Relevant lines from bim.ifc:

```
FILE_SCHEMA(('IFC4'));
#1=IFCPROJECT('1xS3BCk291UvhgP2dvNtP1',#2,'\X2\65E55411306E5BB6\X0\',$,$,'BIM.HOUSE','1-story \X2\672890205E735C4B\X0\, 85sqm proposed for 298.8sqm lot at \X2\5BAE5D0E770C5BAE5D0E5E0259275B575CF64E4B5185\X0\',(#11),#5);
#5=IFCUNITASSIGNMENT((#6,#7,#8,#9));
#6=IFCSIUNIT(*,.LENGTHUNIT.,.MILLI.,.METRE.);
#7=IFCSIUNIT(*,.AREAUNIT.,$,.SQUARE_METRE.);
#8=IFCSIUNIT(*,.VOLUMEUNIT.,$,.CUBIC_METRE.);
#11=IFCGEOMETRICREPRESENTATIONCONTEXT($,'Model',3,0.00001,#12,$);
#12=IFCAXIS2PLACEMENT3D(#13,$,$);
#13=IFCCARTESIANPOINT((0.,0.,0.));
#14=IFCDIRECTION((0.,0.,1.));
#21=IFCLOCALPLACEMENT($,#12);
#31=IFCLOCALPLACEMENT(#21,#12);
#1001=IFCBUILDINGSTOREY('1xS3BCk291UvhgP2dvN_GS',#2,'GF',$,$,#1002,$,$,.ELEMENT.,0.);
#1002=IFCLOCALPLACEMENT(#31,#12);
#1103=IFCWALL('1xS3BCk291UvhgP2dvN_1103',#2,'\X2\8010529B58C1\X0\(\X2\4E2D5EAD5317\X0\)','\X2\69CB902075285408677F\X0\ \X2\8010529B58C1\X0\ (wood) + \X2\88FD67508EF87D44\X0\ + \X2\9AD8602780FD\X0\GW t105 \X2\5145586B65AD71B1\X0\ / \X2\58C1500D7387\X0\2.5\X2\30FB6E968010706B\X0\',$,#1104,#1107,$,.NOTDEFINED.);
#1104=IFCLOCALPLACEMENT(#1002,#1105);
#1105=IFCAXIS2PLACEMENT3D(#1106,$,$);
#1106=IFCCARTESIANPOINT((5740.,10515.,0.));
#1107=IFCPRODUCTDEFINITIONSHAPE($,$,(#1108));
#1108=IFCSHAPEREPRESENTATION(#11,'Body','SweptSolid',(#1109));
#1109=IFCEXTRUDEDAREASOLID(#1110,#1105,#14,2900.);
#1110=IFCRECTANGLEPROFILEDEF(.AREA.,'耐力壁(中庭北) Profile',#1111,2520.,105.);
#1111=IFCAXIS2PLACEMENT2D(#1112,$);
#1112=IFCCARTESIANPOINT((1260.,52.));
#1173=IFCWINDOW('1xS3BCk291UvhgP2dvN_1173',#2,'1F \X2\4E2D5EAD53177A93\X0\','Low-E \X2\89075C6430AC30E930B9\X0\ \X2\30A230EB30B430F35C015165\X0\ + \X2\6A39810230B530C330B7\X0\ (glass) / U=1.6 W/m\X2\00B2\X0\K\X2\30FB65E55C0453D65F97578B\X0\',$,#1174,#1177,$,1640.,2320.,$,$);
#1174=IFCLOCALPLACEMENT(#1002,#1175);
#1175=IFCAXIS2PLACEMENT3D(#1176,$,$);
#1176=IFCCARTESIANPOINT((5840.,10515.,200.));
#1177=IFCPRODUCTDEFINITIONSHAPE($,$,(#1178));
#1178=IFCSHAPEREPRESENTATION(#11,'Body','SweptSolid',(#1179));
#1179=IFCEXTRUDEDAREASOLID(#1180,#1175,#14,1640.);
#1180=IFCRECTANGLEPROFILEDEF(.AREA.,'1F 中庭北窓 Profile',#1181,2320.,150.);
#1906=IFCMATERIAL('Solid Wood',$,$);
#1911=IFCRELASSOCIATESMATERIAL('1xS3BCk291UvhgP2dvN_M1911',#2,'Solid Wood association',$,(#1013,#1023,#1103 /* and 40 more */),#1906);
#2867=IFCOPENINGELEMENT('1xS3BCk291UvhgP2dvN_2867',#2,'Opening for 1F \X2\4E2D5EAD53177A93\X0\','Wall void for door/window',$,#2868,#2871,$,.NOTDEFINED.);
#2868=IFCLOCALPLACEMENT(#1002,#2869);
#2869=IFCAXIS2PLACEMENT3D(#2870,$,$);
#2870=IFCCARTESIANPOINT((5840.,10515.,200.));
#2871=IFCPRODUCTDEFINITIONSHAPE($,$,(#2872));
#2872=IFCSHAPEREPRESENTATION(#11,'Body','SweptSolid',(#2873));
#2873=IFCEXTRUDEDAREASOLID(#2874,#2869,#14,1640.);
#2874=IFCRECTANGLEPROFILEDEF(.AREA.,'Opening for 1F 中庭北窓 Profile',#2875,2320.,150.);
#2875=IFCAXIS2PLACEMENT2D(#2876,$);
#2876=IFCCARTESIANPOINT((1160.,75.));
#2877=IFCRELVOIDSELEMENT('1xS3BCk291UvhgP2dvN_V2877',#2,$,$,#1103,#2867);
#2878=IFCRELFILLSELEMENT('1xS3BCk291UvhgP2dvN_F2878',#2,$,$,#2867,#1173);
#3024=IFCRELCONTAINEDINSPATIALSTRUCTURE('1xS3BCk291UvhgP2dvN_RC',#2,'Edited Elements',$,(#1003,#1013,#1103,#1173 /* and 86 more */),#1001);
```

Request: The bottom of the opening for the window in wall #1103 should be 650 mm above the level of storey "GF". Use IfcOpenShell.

```python
import numpy as np
import ifcopenshell
import ifcopenshell.api.geometry
import ifcopenshell.geom
import ifcopenshell.util.element
import ifcopenshell.util.placement
import ifcopenshell.util.shape
import ifcopenshell.util.unit

model = ifcopenshell.open("bim.ifc")
unit_scale = ifcopenshell.util.unit.calculate_unit_scale(model)

window = model.by_guid("1xS3BCk291UvhgP2dvN_1173")
opening = window.FillsVoids[0].RelatingOpeningElement
storey = ifcopenshell.util.element.get_container(window, ifc_class="IfcBuildingStorey")
level = ifcopenshell.util.placement.get_local_placement(storey.ObjectPlacement)[2, 3]

# The opening's origin need not be at the sill, so measure its lowest point.
shape = ifcopenshell.geom.create_shape(ifcopenshell.geom.settings(), opening)
bottom = ifcopenshell.util.shape.get_shape_bottom_elevation(shape, shape.geometry) / unit_scale
dz = level + 0.65 / unit_scale - bottom

shift = np.array([0.0, 0.0, dz])
# The window is not placed relative to its opening, so move both.
for product in (opening, window):
    matrix = ifcopenshell.util.placement.get_local_placement(product.ObjectPlacement)
    matrix[:3, 3] += shift
    ifcopenshell.api.geometry.edit_object_placement(model, product=product, matrix=matrix, is_si=False)

print(f"moved by {dz * unit_scale:+.3f} m")

model.write("bim_updated.ifc")
```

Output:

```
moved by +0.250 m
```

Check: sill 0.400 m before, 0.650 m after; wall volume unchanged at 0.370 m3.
